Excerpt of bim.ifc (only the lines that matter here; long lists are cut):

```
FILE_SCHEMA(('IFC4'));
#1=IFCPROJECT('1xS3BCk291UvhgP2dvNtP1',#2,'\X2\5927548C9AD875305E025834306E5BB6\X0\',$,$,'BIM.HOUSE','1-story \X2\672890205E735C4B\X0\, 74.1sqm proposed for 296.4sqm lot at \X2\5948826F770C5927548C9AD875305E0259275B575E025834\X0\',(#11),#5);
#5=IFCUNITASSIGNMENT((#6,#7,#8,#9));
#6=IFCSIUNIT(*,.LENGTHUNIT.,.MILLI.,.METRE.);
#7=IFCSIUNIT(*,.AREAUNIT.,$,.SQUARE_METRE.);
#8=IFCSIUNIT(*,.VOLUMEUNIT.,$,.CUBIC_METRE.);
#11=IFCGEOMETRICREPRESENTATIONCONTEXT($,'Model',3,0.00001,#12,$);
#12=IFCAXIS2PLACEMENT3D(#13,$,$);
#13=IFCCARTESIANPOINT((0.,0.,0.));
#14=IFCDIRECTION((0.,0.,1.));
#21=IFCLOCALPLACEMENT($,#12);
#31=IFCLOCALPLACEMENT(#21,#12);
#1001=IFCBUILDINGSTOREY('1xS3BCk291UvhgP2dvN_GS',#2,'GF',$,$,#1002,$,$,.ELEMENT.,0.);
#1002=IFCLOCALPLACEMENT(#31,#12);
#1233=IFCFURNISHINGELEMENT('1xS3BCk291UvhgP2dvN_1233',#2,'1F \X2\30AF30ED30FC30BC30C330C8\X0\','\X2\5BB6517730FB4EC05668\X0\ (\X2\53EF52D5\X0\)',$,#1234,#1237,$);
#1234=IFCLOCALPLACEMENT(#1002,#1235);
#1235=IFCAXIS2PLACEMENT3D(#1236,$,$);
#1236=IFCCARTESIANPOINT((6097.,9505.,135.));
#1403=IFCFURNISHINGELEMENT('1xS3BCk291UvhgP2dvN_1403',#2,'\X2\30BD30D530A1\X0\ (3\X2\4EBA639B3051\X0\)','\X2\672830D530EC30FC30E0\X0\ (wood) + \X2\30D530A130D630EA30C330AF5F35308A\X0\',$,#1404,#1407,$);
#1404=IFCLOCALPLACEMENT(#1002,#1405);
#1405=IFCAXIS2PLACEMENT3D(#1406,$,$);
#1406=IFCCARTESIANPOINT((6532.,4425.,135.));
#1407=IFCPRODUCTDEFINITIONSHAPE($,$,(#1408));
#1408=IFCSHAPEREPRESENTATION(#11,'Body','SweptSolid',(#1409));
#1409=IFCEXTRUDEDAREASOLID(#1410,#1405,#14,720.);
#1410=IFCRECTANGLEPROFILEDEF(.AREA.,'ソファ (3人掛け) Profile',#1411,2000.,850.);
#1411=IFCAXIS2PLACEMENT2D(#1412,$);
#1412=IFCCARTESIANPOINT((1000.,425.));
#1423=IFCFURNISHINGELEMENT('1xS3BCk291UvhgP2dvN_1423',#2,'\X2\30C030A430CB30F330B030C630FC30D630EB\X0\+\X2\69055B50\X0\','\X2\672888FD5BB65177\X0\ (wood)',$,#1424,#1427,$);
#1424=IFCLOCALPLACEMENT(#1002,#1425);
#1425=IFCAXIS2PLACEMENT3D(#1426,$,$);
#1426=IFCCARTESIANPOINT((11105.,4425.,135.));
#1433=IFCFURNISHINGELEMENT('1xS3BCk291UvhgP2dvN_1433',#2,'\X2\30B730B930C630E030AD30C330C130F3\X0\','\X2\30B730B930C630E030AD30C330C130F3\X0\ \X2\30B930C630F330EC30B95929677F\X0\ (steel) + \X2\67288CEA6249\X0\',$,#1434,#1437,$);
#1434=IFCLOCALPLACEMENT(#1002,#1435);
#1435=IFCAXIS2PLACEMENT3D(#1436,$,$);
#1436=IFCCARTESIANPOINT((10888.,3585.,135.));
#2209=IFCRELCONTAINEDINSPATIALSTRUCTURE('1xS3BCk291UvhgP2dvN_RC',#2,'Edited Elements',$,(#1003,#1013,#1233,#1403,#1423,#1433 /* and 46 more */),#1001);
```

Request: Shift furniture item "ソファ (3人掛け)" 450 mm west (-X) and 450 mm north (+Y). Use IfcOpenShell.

```python
import ifcopenshell
import ifcopenshell.api.geometry
import ifcopenshell.util.placement
import ifcopenshell.util.unit

model = ifcopenshell.open("bim.ifc")
unit_scale = ifcopenshell.util.unit.calculate_unit_scale(model)

item = model.by_guid("1xS3BCk291UvhgP2dvN_1403")
matrix = ifcopenshell.util.placement.get_local_placement(item.ObjectPlacement)
matrix[0, 3] -= 0.45 / unit_scale
matrix[1, 3] += 0.45 / unit_scale
ifcopenshell.api.geometry.edit_object_placement(model, product=item, matrix=matrix, is_si=False)

print(ifcopenshell.util.placement.get_local_placement(item.ObjectPlacement).round(3) + 0.0)

model.write("bim-out.ifc")
```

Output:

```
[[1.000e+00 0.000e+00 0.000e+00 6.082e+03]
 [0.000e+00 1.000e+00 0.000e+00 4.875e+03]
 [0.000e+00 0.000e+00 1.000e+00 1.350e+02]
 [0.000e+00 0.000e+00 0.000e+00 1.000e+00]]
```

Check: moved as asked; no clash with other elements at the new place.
